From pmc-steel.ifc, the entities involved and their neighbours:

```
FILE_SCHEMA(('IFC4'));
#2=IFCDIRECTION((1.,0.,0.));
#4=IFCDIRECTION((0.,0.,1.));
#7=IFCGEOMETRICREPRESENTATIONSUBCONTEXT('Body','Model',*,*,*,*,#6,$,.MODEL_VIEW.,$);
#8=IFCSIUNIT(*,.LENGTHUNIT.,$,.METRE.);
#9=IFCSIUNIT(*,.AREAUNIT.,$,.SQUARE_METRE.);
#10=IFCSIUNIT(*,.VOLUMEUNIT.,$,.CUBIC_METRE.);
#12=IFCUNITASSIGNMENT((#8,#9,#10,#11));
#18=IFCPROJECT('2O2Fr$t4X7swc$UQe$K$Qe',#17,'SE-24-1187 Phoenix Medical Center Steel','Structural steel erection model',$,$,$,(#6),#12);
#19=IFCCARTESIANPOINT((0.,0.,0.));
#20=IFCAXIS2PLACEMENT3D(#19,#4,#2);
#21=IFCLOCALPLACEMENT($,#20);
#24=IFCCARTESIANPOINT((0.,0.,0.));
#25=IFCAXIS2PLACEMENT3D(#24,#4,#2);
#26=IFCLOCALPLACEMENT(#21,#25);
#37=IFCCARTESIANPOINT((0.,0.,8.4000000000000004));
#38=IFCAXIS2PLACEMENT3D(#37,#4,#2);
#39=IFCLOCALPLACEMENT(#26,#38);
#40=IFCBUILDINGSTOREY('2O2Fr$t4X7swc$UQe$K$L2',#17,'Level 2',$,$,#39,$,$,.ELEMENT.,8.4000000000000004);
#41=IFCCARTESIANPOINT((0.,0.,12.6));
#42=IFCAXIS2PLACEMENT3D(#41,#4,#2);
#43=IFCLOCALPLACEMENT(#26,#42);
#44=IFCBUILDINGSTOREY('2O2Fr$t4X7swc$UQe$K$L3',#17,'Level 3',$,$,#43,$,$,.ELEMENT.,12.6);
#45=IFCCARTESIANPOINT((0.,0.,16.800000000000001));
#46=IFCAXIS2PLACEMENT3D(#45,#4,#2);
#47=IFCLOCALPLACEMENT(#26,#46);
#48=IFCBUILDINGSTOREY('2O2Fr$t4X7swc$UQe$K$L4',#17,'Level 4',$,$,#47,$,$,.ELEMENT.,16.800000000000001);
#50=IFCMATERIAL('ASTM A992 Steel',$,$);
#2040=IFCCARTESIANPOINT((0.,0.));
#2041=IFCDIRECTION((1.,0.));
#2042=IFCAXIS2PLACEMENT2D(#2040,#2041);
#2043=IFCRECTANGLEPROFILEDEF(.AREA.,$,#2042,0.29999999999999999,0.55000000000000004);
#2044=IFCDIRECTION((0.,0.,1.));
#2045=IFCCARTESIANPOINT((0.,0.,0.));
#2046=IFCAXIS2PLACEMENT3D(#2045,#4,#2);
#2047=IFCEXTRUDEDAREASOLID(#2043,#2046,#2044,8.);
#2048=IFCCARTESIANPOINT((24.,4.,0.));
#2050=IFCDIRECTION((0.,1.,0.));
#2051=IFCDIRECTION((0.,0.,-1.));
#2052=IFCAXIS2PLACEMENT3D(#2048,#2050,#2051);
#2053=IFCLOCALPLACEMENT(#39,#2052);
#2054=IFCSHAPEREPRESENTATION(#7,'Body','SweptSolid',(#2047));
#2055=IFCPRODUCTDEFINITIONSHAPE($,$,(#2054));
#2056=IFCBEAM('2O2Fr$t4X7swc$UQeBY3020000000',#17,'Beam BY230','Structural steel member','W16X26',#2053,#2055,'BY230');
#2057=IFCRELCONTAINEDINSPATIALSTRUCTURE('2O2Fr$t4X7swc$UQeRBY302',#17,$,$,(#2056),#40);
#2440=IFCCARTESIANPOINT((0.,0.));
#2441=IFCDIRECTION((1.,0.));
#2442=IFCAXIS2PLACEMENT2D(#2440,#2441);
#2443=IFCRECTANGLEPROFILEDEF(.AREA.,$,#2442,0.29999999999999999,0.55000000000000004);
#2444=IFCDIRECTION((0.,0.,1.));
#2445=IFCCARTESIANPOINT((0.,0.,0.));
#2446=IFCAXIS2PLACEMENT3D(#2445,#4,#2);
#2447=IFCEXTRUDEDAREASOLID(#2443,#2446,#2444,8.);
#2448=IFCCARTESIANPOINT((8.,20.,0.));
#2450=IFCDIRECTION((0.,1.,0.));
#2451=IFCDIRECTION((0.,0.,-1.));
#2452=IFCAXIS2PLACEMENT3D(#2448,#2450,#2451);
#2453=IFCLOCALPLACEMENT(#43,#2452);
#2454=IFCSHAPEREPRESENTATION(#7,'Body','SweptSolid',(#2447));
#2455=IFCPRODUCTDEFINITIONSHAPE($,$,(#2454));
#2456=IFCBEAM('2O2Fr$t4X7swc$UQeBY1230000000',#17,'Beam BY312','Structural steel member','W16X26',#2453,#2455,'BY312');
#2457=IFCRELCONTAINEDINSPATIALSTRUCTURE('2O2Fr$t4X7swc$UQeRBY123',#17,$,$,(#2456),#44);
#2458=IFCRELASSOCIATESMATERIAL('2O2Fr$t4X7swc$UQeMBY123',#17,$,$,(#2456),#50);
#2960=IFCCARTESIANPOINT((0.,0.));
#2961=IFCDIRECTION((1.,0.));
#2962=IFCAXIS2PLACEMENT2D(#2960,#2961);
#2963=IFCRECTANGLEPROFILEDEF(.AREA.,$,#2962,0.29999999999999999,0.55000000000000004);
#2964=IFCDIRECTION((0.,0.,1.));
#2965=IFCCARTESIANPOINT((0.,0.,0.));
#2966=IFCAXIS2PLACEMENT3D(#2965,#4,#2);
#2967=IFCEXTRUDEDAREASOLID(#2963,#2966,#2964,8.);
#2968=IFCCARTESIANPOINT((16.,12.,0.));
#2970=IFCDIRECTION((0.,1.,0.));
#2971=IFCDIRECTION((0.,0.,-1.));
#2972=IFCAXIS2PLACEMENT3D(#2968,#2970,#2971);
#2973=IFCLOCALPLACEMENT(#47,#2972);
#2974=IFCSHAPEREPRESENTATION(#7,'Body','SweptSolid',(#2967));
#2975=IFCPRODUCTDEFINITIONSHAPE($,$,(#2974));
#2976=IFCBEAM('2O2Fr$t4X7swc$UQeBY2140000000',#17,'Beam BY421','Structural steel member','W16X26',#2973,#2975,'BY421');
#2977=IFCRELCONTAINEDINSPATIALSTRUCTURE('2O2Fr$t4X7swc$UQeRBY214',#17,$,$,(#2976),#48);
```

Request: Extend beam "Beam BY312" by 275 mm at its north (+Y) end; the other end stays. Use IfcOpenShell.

```python
import ifcopenshell
import ifcopenshell.util.representation

model = ifcopenshell.open("pmc-steel.ifc")

member = model.by_guid("2O2Fr$t4X7swc$UQeBY1230000000")
change = 0.275

# The extrusion runs towards the end named, so only its depth changes.
body = ifcopenshell.util.representation.get_representation(member, "Model", "Body")
solid = body.Items[0]
old_length = solid.Depth
solid.Depth += change

print(f"length {old_length:g} -> {solid.Depth:g}")

model.write("pmc-steel_updated.ifc")
```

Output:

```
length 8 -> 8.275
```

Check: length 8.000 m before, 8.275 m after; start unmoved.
